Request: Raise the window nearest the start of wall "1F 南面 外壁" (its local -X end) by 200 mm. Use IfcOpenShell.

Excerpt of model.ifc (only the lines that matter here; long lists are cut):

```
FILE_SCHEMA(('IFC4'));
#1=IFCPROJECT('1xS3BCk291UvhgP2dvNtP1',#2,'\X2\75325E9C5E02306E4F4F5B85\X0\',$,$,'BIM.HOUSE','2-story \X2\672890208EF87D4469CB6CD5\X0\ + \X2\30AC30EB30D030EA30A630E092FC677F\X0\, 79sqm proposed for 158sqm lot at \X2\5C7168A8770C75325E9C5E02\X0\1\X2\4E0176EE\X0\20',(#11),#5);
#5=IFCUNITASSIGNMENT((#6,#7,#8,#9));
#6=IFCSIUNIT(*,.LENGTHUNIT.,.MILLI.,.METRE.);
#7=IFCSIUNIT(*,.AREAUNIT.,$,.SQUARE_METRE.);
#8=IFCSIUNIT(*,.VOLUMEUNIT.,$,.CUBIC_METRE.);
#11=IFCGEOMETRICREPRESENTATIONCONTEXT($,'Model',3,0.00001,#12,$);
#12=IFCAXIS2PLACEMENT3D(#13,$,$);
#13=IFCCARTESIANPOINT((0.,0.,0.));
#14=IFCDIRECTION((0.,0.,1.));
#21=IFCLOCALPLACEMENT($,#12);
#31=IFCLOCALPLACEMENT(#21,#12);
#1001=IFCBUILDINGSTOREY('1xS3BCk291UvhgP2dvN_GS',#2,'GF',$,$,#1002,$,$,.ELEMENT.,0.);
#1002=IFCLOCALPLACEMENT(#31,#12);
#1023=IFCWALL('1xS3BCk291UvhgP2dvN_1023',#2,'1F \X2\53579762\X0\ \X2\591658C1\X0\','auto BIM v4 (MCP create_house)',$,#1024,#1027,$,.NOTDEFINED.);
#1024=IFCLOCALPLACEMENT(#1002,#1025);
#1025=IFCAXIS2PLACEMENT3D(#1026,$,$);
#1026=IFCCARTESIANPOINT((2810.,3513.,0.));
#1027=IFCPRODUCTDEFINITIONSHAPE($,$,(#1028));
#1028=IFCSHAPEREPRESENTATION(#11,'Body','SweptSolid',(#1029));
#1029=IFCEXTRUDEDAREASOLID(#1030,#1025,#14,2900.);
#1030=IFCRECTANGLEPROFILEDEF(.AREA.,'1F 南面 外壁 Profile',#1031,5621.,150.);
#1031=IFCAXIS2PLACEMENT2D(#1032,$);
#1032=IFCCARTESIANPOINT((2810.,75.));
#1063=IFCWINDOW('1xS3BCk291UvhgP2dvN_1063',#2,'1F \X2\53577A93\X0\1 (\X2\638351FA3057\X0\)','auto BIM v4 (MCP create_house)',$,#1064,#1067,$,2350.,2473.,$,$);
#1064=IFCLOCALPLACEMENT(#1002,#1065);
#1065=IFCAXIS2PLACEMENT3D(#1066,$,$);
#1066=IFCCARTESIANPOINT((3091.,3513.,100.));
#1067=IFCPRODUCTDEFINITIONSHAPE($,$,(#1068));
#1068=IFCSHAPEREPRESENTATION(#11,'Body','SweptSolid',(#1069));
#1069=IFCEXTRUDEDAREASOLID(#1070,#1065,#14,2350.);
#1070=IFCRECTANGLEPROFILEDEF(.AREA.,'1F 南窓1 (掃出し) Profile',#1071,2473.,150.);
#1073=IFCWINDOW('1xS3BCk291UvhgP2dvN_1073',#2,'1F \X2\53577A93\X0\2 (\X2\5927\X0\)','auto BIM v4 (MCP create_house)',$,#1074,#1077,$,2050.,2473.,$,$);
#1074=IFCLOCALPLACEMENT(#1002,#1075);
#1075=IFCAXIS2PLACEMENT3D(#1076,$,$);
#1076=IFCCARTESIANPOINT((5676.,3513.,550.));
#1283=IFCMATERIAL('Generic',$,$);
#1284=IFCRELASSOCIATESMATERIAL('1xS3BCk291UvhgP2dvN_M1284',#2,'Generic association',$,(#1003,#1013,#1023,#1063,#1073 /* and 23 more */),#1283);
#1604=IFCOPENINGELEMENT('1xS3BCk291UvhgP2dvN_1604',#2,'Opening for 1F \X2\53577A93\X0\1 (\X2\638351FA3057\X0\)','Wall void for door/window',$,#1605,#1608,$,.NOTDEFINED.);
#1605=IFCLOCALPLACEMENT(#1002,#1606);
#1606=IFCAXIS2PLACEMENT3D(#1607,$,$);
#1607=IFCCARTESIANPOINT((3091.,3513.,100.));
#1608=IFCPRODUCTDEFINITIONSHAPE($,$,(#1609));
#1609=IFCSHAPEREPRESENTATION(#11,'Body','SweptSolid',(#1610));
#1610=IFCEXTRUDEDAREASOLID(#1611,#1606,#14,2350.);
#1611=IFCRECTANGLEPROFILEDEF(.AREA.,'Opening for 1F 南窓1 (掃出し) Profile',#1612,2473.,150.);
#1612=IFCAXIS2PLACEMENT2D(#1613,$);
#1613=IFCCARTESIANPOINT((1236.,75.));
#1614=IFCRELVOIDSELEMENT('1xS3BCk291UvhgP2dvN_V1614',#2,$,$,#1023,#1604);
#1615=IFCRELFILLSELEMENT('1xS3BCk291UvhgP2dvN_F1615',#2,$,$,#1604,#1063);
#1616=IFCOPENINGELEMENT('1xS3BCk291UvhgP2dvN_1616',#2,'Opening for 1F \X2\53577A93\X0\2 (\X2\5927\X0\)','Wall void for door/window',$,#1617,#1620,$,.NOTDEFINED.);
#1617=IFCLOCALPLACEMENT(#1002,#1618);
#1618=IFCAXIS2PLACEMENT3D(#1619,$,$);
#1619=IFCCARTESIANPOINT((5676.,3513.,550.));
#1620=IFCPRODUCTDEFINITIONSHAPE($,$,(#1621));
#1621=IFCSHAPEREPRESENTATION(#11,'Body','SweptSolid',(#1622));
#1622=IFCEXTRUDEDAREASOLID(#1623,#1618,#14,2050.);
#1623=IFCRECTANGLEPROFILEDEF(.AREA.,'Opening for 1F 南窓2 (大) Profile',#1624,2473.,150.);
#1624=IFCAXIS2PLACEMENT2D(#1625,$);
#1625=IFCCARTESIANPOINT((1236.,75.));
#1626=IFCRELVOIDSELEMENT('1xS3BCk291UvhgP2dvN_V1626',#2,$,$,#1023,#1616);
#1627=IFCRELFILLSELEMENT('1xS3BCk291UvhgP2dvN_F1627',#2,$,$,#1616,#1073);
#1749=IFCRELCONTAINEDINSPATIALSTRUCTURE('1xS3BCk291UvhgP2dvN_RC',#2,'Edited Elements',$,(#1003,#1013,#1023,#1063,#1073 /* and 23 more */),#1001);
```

```python
import numpy as np
import ifcopenshell
import ifcopenshell.api.geometry
import ifcopenshell.util.placement
import ifcopenshell.util.unit

model = ifcopenshell.open("model.ifc")
unit_scale = ifcopenshell.util.unit.calculate_unit_scale(model)

window = model.by_guid("1xS3BCk291UvhgP2dvN_1063")
opening = window.FillsVoids[0].RelatingOpeningElement
dz = 0.2 / unit_scale

shift = np.array([0.0, 0.0, dz])
# The window is not placed relative to its opening, so move both.
for product in (opening, window):
    matrix = ifcopenshell.util.placement.get_local_placement(product.ObjectPlacement)
    matrix[:3, 3] += shift
    ifcopenshell.api.geometry.edit_object_placement(model, product=product, matrix=matrix, is_si=False)

print(f"moved by {dz * unit_scale:+.3f} m")

model.write("model_v2.ifc")
```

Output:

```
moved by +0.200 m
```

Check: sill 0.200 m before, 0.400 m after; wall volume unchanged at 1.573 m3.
